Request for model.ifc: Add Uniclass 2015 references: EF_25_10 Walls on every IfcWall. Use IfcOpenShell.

First a look at what the model holds.

```python
import ifcopenshell

model = ifcopenshell.open("model.ifc")
print(model.schema)
print("classifications:", [c.Name for c in model.by_type("IfcClassification")])
for ifc_class in ("IfcDoor", "IfcRoof", "IfcStair", "IfcWall", "IfcWindow"):
    print(ifc_class, len(model.by_type(ifc_class)))
```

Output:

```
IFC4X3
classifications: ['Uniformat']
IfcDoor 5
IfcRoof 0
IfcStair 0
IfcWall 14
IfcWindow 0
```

```python
import ifcopenshell
import ifcopenshell.api.classification

model = ifcopenshell.open("model.ifc")

system = ifcopenshell.api.classification.add_classification(model, classification="Uniclass 2015")

codes = {
    "IfcWall": ("EF_25_10", "Walls"),
}
for ifc_class, (code, name) in codes.items():
    products = model.by_type(ifc_class)
    ifcopenshell.api.classification.add_reference(
        model, products=products, classification=system, identification=code, name=name
    )
    print(code, len(products))

model.write("model_edited.ifc")
```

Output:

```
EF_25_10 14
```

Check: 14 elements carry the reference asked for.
